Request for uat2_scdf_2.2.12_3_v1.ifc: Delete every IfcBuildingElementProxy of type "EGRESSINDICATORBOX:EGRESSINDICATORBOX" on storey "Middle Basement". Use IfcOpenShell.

First a look at what the model holds.

```python
import ifcopenshell
import ifcopenshell.util.element

model = ifcopenshell.open("uat2_scdf_2.2.12_3_v1.ifc")
print(model.schema)
storey = next(s for s in model.by_type("IfcBuildingStorey") if s.Name == "Middle Basement")
proxies = [e for e in ifcopenshell.util.element.get_decomposition(storey) if e.is_a("IfcBuildingElementProxy")]
seen = {}
for e in proxies:
    element_type = ifcopenshell.util.element.get_type(e)
    name = element_type.Name if element_type not in (None, e) else None
    seen[name] = seen.get(name, 0) + 1
for name, count in sorted(seen.items(), key=str):
    print(count, "x", name)
```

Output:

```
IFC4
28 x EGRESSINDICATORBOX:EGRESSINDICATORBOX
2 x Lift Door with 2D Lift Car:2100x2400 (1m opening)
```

```python
import ifcopenshell
import ifcopenshell.api.root
import ifcopenshell.util.element

model = ifcopenshell.open("uat2_scdf_2.2.12_3_v1.ifc")

storey = next(s for s in model.by_type("IfcBuildingStorey") if s.Name == "Middle Basement")
proxies = [e for e in ifcopenshell.util.element.get_decomposition(storey) if e.is_a("IfcBuildingElementProxy")]
targets = [e for e in proxies if (t := ifcopenshell.util.element.get_type(e)) not in (None, e) and t.Name == "EGRESSINDICATORBOX:EGRESSINDICATORBOX"]

for e in targets:
    ifcopenshell.api.root.remove_product(model, product=e)
print(len(targets), "removed")

model.write("uat2_scdf_2.2.12_3_v1-out.ifc")
```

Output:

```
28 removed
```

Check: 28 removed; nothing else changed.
